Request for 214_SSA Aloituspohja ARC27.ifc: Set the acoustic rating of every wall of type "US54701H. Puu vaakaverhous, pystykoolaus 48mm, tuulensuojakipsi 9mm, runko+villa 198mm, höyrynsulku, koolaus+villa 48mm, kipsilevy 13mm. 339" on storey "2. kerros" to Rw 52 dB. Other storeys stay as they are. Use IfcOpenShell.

First a look at what the model holds.

```python
import ifcopenshell
import ifcopenshell.util.element

model = ifcopenshell.open("214_SSA Aloituspohja ARC27.ifc")
print(model.schema)
storey = next(s for s in model.by_type("IfcBuildingStorey") if s.Name == "2. kerros")
walls = [e for e in ifcopenshell.util.element.get_decomposition(storey) if e.is_a("IfcWall")]
seen = {}
for e in walls:
    element_type = ifcopenshell.util.element.get_type(e)
    key = (element_type.Name if element_type != e and element_type else None, ifcopenshell.util.element.get_pset(e, "Pset_WallCommon", "AcousticRating"))
    seen[key] = seen.get(key, 0) + 1
for (name, value), count in sorted(seen.items(), key=str):
    print(count, "x", name, "|", value)
```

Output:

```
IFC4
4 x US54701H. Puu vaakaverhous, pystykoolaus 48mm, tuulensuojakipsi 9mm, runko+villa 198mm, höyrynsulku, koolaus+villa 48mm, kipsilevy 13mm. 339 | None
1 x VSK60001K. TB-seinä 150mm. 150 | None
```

```python
import ifcopenshell
import ifcopenshell.api.pset
import ifcopenshell.util.element

model = ifcopenshell.open("214_SSA Aloituspohja ARC27.ifc")

storey = next(s for s in model.by_type("IfcBuildingStorey") if s.Name == "2. kerros")
walls = [e for e in ifcopenshell.util.element.get_decomposition(storey) if e.is_a("IfcWall")]

count = 0
for e in walls:
    element_type = ifcopenshell.util.element.get_type(e)
    if element_type in (None, e) or element_type.Name != "US54701H. Puu vaakaverhous, pystykoolaus 48mm, tuulensuojakipsi 9mm, runko+villa 198mm, höyrynsulku, koolaus+villa 48mm, kipsilevy 13mm. 339":
        continue
    # add_pset returns the element's existing set when there is one.
    pset = ifcopenshell.api.pset.add_pset(model, product=e, name="Pset_WallCommon")
    ifcopenshell.api.pset.edit_pset(model, pset=pset, properties={"AcousticRating": "Rw 52 dB"})
    count += 1

print(count, "walls updated")

model.write("214_SSA Aloituspohja ARC27_edited.ifc")
```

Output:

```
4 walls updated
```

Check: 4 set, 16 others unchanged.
